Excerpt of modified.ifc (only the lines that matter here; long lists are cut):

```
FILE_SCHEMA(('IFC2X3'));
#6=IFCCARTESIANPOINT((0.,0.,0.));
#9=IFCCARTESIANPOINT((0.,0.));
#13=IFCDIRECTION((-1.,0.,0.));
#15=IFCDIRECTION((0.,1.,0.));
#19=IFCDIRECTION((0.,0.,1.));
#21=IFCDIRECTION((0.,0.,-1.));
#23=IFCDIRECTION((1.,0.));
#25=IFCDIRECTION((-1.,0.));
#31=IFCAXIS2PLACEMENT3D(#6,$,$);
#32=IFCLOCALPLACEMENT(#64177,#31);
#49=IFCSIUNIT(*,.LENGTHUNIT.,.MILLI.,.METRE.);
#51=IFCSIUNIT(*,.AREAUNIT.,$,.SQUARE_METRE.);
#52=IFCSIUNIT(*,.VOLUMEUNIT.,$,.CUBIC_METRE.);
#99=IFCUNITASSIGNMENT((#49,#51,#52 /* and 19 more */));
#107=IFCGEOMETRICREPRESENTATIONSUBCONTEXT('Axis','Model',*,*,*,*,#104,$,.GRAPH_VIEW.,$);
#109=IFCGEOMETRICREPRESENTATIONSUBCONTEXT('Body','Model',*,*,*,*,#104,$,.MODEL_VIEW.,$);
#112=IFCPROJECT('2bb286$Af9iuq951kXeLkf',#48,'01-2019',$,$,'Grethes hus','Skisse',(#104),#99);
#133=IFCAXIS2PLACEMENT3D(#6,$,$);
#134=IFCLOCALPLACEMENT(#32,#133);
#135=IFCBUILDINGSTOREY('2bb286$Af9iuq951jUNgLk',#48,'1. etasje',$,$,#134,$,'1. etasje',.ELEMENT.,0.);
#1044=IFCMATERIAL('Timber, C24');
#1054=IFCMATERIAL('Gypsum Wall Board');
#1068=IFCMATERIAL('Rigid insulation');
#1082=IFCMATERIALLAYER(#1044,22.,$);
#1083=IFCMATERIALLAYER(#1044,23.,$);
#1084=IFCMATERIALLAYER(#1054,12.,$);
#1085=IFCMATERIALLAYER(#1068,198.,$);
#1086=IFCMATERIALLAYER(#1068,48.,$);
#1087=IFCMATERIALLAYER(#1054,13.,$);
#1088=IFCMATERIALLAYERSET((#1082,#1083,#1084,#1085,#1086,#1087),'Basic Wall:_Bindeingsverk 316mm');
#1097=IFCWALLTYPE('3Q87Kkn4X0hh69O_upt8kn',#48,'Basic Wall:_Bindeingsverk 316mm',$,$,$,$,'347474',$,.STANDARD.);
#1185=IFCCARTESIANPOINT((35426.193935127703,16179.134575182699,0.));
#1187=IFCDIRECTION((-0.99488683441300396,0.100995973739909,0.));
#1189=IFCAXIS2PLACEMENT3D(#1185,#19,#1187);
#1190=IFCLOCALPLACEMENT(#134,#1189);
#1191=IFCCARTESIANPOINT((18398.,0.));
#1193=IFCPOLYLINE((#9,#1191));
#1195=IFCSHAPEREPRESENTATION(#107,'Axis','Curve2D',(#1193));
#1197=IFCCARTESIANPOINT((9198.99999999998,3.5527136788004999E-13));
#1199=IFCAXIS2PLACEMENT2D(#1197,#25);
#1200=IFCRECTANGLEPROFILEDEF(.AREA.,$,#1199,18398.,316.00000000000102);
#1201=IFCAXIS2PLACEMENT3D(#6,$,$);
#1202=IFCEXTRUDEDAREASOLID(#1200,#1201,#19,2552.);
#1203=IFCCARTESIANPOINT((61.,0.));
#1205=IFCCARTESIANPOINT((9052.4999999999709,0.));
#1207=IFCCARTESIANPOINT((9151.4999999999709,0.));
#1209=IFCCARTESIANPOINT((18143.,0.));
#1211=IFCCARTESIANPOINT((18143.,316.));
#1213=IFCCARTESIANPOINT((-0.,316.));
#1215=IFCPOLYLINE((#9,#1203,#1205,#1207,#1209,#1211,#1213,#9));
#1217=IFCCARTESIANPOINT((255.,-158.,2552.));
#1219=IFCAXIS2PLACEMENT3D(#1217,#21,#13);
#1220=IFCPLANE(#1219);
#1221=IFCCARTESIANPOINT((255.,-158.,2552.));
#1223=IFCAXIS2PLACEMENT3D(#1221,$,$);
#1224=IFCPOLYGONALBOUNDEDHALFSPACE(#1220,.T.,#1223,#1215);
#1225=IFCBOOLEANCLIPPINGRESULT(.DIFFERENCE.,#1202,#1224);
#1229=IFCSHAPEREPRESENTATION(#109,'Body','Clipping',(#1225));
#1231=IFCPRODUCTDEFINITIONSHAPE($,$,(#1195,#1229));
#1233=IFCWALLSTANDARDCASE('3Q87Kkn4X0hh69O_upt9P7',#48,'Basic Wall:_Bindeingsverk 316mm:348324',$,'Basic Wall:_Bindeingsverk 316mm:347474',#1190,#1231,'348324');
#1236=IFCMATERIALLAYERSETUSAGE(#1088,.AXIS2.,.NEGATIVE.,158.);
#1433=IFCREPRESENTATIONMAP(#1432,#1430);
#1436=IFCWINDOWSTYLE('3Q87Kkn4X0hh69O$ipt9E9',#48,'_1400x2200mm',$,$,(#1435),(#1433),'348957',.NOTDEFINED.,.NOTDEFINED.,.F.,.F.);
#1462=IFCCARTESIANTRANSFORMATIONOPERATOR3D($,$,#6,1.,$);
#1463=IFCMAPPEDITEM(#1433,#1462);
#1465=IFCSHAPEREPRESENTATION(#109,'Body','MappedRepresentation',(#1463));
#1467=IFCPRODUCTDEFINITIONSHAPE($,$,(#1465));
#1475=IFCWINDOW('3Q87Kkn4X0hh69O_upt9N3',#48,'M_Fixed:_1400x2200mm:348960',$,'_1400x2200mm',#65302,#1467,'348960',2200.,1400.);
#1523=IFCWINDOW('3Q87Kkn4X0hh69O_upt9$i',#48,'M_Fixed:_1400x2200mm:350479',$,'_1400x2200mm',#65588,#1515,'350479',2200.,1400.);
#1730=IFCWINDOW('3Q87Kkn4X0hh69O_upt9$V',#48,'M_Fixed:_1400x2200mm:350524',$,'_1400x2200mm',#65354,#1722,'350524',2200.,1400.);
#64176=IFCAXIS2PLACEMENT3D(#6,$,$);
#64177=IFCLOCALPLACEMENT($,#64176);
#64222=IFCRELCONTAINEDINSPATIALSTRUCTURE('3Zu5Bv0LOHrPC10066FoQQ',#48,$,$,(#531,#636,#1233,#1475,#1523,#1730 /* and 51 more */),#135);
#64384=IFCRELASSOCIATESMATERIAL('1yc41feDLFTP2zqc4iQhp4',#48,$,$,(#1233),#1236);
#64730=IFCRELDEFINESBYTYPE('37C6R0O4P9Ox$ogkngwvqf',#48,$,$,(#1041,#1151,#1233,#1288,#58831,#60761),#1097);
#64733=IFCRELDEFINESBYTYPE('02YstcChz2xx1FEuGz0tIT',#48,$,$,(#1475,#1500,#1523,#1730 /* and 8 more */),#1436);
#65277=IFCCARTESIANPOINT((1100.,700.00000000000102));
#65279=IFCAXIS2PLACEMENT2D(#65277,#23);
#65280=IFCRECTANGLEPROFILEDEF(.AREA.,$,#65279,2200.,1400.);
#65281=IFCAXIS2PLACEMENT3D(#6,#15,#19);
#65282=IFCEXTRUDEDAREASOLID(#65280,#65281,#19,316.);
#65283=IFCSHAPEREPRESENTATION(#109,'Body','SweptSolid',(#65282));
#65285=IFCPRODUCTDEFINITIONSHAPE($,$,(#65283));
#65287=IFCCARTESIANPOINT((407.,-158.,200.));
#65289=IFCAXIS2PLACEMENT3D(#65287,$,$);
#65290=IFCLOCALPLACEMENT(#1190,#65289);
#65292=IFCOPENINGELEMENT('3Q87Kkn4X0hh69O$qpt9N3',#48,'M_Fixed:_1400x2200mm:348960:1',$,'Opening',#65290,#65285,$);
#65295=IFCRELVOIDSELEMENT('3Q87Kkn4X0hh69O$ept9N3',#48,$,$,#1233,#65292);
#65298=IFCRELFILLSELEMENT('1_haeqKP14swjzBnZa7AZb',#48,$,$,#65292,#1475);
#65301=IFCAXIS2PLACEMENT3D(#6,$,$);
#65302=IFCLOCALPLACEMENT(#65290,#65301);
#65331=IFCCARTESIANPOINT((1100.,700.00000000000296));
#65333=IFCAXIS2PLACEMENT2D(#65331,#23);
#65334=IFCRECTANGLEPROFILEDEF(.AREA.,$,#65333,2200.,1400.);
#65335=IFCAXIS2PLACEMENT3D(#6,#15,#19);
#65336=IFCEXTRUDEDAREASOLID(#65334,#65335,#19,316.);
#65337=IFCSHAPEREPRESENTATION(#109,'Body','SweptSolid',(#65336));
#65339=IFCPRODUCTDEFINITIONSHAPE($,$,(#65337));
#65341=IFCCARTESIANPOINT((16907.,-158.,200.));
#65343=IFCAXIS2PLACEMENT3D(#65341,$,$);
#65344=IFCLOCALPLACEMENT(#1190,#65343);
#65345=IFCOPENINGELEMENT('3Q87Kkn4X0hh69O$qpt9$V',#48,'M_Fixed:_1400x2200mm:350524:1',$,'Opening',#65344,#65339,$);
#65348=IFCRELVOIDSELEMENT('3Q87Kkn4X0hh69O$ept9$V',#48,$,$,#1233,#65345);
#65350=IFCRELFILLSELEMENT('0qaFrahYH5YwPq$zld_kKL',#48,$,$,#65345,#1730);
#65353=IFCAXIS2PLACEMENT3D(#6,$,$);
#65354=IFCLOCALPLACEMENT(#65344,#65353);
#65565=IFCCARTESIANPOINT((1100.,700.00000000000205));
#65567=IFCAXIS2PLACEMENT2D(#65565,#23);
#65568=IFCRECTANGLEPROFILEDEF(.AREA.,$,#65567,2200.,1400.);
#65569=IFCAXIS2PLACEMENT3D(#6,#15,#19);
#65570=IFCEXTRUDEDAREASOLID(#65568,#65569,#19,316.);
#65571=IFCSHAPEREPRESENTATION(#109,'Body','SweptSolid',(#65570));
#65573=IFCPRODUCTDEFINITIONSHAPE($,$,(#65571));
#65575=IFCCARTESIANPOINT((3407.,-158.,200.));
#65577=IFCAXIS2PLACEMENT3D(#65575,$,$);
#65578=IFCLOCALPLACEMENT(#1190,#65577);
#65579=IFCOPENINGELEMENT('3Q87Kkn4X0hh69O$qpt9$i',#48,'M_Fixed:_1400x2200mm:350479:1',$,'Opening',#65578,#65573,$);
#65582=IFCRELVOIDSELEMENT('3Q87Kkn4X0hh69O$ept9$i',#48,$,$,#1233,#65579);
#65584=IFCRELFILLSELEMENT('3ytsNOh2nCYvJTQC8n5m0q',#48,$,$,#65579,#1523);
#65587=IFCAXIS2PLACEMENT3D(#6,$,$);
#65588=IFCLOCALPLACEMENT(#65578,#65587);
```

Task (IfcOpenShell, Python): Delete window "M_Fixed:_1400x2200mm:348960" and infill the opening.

```python
import ifcopenshell
import ifcopenshell.api.feature
import ifcopenshell.api.root
import ifcopenshell.geom
import ifcopenshell.util.shape

model = ifcopenshell.open("modified.ifc")
settings = ifcopenshell.geom.settings()


def volume(element):
    """Net volume in cubic metres, openings subtracted."""
    shape = ifcopenshell.geom.create_shape(settings, element)
    return ifcopenshell.util.shape.get_volume(shape.geometry)


window = model.by_id(1475)
opening = window.FillsVoids[0].RelatingOpeningElement
wall = opening.VoidsElements[0].RelatingBuildingElement
before = volume(wall)

ifcopenshell.api.root.remove_product(model, product=window)
ifcopenshell.api.feature.remove_feature(model, feature=opening)

after = volume(wall)

print(f"wall volume {before:.3f} -> {after:.3f} m3")

model.write("modified_edited.ifc")
```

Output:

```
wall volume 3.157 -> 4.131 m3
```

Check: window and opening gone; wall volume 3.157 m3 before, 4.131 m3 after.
